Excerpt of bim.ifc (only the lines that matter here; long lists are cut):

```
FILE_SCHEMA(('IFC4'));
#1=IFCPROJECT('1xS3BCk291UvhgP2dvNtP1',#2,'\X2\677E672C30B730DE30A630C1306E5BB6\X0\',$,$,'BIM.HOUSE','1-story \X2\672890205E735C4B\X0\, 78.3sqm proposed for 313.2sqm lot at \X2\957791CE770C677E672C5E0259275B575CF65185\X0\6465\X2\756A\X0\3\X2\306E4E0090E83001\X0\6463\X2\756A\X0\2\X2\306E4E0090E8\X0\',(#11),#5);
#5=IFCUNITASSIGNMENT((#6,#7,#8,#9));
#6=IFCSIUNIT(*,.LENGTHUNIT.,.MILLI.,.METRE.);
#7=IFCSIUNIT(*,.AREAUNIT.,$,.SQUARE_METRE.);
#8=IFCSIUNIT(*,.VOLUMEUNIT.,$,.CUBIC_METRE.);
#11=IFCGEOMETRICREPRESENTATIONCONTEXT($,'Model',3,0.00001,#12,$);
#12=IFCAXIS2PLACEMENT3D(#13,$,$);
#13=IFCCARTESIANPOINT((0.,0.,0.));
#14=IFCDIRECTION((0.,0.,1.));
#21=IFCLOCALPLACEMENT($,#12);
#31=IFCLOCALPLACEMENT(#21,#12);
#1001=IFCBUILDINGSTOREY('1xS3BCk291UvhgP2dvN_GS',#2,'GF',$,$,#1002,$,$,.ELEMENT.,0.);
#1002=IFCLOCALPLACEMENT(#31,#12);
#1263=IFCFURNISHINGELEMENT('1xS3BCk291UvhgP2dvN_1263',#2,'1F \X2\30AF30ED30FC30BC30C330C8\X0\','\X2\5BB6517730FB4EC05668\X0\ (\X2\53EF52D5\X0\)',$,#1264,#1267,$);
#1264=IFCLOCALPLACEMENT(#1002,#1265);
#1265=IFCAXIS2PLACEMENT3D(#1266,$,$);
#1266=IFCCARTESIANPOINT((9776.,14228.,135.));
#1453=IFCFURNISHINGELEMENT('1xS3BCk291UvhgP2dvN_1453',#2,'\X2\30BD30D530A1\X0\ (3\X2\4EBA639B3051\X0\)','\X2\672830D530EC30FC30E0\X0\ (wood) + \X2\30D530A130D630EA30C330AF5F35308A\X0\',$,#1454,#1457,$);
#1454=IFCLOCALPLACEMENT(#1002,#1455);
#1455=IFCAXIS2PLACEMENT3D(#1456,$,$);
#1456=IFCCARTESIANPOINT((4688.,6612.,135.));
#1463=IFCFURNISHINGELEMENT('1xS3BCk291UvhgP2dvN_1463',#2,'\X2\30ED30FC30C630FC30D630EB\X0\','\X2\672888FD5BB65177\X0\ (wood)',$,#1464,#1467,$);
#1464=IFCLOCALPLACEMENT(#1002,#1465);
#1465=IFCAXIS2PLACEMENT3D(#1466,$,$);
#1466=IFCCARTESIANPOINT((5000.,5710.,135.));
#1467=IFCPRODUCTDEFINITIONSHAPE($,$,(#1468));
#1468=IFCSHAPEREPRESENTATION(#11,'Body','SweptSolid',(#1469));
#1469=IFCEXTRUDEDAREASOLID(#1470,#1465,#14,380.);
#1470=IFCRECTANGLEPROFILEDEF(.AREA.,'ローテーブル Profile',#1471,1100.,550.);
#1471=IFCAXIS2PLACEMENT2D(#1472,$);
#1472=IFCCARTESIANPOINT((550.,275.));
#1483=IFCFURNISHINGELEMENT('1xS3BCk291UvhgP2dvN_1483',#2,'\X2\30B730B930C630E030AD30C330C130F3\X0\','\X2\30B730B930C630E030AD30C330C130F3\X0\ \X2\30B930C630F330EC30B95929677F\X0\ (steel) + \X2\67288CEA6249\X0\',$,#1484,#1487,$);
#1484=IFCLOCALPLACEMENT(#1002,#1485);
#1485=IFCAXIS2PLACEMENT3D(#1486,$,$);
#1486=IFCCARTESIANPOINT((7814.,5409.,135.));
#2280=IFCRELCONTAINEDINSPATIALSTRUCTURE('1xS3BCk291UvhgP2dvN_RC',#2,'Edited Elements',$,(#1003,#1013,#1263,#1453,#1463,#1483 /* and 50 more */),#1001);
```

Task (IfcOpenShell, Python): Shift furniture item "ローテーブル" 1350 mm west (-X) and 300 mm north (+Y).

```python
import ifcopenshell
import ifcopenshell.api.geometry
import ifcopenshell.util.placement
import ifcopenshell.util.unit

model = ifcopenshell.open("bim.ifc")
unit_scale = ifcopenshell.util.unit.calculate_unit_scale(model)

item = model.by_id(1463)
matrix = ifcopenshell.util.placement.get_local_placement(item.ObjectPlacement)
matrix[0, 3] -= 1.35 / unit_scale
matrix[1, 3] += 0.3 / unit_scale
ifcopenshell.api.geometry.edit_object_placement(model, product=item, matrix=matrix, is_si=False)

print(ifcopenshell.util.placement.get_local_placement(item.ObjectPlacement).round(3) + 0.0)

model.write("bim-out.ifc")
```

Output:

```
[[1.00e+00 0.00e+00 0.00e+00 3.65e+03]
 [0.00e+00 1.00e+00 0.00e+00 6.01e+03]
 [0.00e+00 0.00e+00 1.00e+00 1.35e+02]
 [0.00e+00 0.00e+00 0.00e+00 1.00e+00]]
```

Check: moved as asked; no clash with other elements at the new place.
